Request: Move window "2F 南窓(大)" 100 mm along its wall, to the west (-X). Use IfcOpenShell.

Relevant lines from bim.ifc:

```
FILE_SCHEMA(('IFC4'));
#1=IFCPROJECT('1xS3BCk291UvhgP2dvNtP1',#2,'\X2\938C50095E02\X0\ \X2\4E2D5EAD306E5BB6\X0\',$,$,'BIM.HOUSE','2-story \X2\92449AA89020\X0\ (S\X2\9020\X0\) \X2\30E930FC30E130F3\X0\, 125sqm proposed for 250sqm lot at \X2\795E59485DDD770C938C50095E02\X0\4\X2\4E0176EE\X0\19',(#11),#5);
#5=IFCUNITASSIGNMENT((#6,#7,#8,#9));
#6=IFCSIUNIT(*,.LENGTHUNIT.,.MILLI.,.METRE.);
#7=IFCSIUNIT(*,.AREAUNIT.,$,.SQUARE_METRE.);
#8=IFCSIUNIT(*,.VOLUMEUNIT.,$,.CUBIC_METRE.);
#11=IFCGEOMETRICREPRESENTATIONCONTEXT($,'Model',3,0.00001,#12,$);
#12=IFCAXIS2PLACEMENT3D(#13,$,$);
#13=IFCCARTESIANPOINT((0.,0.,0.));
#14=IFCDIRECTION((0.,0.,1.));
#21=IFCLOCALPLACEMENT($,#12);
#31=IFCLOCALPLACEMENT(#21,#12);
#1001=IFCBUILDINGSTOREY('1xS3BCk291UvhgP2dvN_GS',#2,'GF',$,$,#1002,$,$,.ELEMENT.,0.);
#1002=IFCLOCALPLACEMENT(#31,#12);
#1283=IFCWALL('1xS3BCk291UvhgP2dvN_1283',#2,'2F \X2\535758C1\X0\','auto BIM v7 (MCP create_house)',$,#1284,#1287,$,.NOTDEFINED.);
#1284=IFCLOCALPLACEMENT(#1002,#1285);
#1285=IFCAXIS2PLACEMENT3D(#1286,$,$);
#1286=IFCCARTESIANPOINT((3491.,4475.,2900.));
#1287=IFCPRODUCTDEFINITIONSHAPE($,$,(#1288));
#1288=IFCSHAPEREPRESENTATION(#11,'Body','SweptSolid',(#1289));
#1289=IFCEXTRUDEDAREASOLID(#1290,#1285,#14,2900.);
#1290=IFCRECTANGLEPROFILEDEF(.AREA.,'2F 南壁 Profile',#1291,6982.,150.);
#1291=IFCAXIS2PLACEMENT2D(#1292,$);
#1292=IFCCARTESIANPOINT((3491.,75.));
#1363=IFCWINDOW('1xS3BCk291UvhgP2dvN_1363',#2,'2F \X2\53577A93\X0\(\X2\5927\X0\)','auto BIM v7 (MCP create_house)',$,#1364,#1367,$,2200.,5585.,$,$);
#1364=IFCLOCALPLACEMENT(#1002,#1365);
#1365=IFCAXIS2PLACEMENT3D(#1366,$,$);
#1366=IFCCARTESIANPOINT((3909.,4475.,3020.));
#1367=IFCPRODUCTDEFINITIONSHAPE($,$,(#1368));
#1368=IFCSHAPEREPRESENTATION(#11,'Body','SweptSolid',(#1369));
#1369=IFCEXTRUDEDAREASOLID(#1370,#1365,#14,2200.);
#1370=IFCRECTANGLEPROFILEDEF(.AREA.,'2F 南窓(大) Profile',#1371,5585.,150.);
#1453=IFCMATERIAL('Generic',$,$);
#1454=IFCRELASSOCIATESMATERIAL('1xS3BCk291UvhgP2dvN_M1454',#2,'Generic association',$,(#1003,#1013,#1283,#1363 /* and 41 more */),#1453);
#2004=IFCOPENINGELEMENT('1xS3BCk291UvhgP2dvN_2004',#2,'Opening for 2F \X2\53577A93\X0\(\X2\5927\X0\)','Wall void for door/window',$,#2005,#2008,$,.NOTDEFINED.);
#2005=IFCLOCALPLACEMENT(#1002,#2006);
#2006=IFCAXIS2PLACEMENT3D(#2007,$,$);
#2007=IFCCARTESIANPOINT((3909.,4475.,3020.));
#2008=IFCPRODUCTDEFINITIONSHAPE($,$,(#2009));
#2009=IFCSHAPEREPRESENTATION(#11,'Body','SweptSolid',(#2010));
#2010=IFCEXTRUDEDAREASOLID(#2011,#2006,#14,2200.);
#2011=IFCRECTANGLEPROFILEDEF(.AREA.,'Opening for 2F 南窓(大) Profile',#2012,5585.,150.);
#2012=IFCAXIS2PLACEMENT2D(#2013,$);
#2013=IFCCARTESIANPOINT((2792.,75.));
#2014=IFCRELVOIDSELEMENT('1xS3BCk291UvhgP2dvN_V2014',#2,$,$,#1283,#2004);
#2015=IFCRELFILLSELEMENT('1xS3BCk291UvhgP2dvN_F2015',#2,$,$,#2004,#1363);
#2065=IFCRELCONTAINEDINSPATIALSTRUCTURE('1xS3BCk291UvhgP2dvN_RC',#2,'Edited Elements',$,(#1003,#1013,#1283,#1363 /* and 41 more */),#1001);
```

```python
import ifcopenshell
import ifcopenshell.api.geometry
import ifcopenshell.util.placement
import ifcopenshell.util.unit

model = ifcopenshell.open("bim.ifc")
unit_scale = ifcopenshell.util.unit.calculate_unit_scale(model)

window = model.by_guid("1xS3BCk291UvhgP2dvN_1363")
opening = window.FillsVoids[0].RelatingOpeningElement
wall = opening.VoidsElements[0].RelatingBuildingElement

wall_matrix = ifcopenshell.util.placement.get_local_placement(wall.ObjectPlacement)
shift = wall_matrix[:3, 0] * -0.1 / unit_scale
before = ifcopenshell.util.placement.get_local_placement(window.ObjectPlacement)[:3, 3].copy()

# The window is not placed relative to its opening, so move both.
for product in (opening, window):
    matrix = ifcopenshell.util.placement.get_local_placement(product.ObjectPlacement)
    matrix[:3, 3] += shift
    ifcopenshell.api.geometry.edit_object_placement(model, product=product, matrix=matrix, is_si=False)

after = ifcopenshell.util.placement.get_local_placement(window.ObjectPlacement)[:3, 3]
print("window moved by", (after - before).round(3) + 0.0)

model.write("bim-out.ifc")
```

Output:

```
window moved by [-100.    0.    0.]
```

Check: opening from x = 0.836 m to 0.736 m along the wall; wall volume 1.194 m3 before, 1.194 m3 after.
